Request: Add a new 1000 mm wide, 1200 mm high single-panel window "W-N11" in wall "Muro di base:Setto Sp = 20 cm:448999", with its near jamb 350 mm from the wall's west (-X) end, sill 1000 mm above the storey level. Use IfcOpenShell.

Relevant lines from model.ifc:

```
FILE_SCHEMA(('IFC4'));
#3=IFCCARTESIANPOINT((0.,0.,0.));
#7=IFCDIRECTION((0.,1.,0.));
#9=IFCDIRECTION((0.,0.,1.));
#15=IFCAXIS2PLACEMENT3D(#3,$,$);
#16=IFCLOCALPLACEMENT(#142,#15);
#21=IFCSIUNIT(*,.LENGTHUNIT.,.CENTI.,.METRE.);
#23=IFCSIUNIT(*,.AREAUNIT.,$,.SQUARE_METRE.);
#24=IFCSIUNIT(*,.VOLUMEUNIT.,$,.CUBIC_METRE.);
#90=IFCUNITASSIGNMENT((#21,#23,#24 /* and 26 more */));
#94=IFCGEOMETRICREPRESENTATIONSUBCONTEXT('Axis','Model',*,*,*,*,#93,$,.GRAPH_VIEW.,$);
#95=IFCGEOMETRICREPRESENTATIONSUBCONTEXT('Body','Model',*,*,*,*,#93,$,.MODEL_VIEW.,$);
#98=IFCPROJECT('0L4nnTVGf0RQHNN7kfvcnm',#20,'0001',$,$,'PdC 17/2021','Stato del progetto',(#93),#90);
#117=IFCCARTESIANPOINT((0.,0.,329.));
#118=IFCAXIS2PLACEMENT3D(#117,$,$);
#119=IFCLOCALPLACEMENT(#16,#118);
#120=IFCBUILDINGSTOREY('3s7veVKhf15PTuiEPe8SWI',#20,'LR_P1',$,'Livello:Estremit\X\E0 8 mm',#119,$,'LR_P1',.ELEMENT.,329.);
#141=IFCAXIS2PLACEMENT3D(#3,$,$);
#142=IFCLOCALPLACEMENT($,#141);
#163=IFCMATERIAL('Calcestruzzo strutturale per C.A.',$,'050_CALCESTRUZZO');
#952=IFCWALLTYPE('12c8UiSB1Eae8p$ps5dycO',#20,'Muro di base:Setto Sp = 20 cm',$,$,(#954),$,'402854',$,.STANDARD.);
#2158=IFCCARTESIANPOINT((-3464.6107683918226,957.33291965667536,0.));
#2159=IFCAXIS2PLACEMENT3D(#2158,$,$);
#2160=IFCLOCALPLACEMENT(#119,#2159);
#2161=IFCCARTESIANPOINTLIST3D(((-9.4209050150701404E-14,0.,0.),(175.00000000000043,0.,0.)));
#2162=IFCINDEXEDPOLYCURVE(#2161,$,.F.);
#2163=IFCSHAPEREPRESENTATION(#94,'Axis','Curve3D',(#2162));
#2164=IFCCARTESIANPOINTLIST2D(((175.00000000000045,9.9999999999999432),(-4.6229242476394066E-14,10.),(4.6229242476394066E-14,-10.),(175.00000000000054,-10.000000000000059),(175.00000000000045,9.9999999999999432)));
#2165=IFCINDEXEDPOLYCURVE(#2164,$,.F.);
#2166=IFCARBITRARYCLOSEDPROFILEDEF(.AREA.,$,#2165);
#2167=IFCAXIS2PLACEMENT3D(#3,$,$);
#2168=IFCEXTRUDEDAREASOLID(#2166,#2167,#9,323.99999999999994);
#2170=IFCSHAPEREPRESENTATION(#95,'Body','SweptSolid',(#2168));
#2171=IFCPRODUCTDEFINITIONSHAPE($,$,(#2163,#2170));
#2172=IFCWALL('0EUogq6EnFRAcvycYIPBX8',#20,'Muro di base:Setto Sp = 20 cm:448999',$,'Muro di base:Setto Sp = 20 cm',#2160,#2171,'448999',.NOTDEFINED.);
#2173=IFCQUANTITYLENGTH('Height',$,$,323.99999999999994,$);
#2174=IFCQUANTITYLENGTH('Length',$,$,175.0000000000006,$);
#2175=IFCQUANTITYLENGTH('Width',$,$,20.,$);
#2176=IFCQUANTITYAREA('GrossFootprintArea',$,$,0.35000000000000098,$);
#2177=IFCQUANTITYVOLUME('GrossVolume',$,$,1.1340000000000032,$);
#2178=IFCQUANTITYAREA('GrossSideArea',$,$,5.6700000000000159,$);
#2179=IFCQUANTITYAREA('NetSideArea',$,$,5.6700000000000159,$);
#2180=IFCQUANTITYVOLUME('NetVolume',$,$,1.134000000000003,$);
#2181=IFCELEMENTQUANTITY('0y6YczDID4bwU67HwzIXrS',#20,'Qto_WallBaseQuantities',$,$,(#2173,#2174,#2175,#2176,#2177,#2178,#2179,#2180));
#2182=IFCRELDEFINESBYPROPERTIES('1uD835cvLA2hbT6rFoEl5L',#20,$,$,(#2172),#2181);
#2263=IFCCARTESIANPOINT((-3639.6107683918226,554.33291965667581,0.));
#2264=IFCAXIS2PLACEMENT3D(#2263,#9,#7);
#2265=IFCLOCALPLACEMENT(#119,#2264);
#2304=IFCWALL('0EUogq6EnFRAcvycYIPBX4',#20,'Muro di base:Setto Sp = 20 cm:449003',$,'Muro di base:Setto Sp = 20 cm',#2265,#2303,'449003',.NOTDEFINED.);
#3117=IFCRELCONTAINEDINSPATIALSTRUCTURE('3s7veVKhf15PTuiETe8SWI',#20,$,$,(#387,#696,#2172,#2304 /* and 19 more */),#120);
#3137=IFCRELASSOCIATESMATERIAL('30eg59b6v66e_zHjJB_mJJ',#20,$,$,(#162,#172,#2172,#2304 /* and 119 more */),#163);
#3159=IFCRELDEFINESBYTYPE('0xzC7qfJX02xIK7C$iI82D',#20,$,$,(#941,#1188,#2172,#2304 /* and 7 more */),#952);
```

```python
import numpy as np
import ifcopenshell
import ifcopenshell.api.feature
import ifcopenshell.api.geometry
import ifcopenshell.api.pset
import ifcopenshell.api.root
import ifcopenshell.api.spatial
import ifcopenshell.geom
import ifcopenshell.util.element
import ifcopenshell.util.placement
import ifcopenshell.util.representation
import ifcopenshell.util.shape
import ifcopenshell.util.unit

model = ifcopenshell.open("model.ifc")
unit_scale = ifcopenshell.util.unit.calculate_unit_scale(model)
area_scale = ifcopenshell.util.unit.calculate_unit_scale(model, "AREAUNIT")
volume_scale = ifcopenshell.util.unit.calculate_unit_scale(model, "VOLUMEUNIT")
settings = ifcopenshell.geom.settings()


def volume(element):
    """Net volume in cubic metres, openings subtracted."""
    shape = ifcopenshell.geom.create_shape(settings, element)
    return ifcopenshell.util.shape.get_volume(shape.geometry)


wall = model.by_id(2172)
storey = ifcopenshell.util.element.get_container(wall, ifc_class="IfcBuildingStorey")
context = ifcopenshell.util.representation.get_context(model, "Model", "Body", "MODEL_VIEW")
before = volume(wall)

width, height, from_end, sill = 1, 1.2, 0.35, 1  # metres

# The wall runs along its own X axis, and the end named is its -X end.
wall_shape = ifcopenshell.geom.create_shape(settings, wall)
x, y, z = ifcopenshell.util.shape.get_vertices(wall_shape.geometry).T
start = x.min() + from_end
face, thickness = float(y.min()), float(y.max() - y.min())
wall_matrix = ifcopenshell.util.placement.get_local_placement(wall.ObjectPlacement)
level = ifcopenshell.util.placement.get_local_placement(storey.ObjectPlacement)[2, 3]


def in_wall(x, y):
    """Placement at x, y metres in the wall's axes, at sill height."""
    matrix = wall_matrix.copy()
    matrix[:, 3] = wall_matrix @ np.array([x / unit_scale, y / unit_scale, 0.0, 1.0])
    matrix[2, 3] = level + sill / unit_scale
    return matrix


# Opening: a box that overshoots both wall faces by 50 mm.
opening = ifcopenshell.api.root.create_entity(model, ifc_class="IfcOpeningElement", predefined_type="OPENING")
box = ifcopenshell.api.geometry.add_wall_representation(
    model, context=context, length=width, height=height, thickness=thickness + 0.1
)
ifcopenshell.api.geometry.assign_representation(model, product=opening, representation=box)
ifcopenshell.api.geometry.edit_object_placement(model, product=opening, matrix=in_wall(start, face - 0.05), is_si=False)
ifcopenshell.api.feature.add_feature(model, feature=opening, element=wall)

window = ifcopenshell.api.root.create_entity(model, ifc_class="IfcWindow", name="W-N11", predefined_type="WINDOW")
window.OverallWidth, window.OverallHeight = width / unit_scale, height / unit_scale
window.PartitioningType = "SINGLE_PANEL"
body = ifcopenshell.api.geometry.add_window_representation(
    model,
    context=context,
    overall_width=window.OverallWidth,
    overall_height=window.OverallHeight,
    partition_type="SINGLE_PANEL",
)
ifcopenshell.api.geometry.assign_representation(model, product=window, representation=body)
ifcopenshell.api.spatial.assign_container(model, products=[window], relating_structure=storey)
ifcopenshell.api.feature.add_filling(model, opening=opening, element=window)

# Centre the window in the wall's thickness.
ifcopenshell.api.geometry.edit_object_placement(model, product=window, matrix=in_wall(start, face), is_si=False)
window_shape = ifcopenshell.geom.create_shape(settings, window)
depth = ifcopenshell.util.shape.get_vertices(window_shape.geometry)[:, 1]
offset = face + thickness / 2 - (depth.min() + depth.max()) / 2
ifcopenshell.api.geometry.edit_object_placement(model, product=window, matrix=in_wall(start, offset), is_si=False)

after = volume(wall)

# Update the wall's stored quantities.
qto = model.by_id(ifcopenshell.util.element.get_pset(wall, "Qto_WallBaseQuantities", should_inherit=False)["id"])
ifcopenshell.api.pset.edit_qto(model, qto=qto, properties={
    "NetSideArea": after / thickness / area_scale,
    "NetVolume": after / volume_scale,
})

print(f"wall volume {before:.3f} -> {after:.3f} m3")

model.write("model_edited.ifc")
```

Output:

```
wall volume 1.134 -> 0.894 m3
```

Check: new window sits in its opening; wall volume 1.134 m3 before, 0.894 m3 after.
